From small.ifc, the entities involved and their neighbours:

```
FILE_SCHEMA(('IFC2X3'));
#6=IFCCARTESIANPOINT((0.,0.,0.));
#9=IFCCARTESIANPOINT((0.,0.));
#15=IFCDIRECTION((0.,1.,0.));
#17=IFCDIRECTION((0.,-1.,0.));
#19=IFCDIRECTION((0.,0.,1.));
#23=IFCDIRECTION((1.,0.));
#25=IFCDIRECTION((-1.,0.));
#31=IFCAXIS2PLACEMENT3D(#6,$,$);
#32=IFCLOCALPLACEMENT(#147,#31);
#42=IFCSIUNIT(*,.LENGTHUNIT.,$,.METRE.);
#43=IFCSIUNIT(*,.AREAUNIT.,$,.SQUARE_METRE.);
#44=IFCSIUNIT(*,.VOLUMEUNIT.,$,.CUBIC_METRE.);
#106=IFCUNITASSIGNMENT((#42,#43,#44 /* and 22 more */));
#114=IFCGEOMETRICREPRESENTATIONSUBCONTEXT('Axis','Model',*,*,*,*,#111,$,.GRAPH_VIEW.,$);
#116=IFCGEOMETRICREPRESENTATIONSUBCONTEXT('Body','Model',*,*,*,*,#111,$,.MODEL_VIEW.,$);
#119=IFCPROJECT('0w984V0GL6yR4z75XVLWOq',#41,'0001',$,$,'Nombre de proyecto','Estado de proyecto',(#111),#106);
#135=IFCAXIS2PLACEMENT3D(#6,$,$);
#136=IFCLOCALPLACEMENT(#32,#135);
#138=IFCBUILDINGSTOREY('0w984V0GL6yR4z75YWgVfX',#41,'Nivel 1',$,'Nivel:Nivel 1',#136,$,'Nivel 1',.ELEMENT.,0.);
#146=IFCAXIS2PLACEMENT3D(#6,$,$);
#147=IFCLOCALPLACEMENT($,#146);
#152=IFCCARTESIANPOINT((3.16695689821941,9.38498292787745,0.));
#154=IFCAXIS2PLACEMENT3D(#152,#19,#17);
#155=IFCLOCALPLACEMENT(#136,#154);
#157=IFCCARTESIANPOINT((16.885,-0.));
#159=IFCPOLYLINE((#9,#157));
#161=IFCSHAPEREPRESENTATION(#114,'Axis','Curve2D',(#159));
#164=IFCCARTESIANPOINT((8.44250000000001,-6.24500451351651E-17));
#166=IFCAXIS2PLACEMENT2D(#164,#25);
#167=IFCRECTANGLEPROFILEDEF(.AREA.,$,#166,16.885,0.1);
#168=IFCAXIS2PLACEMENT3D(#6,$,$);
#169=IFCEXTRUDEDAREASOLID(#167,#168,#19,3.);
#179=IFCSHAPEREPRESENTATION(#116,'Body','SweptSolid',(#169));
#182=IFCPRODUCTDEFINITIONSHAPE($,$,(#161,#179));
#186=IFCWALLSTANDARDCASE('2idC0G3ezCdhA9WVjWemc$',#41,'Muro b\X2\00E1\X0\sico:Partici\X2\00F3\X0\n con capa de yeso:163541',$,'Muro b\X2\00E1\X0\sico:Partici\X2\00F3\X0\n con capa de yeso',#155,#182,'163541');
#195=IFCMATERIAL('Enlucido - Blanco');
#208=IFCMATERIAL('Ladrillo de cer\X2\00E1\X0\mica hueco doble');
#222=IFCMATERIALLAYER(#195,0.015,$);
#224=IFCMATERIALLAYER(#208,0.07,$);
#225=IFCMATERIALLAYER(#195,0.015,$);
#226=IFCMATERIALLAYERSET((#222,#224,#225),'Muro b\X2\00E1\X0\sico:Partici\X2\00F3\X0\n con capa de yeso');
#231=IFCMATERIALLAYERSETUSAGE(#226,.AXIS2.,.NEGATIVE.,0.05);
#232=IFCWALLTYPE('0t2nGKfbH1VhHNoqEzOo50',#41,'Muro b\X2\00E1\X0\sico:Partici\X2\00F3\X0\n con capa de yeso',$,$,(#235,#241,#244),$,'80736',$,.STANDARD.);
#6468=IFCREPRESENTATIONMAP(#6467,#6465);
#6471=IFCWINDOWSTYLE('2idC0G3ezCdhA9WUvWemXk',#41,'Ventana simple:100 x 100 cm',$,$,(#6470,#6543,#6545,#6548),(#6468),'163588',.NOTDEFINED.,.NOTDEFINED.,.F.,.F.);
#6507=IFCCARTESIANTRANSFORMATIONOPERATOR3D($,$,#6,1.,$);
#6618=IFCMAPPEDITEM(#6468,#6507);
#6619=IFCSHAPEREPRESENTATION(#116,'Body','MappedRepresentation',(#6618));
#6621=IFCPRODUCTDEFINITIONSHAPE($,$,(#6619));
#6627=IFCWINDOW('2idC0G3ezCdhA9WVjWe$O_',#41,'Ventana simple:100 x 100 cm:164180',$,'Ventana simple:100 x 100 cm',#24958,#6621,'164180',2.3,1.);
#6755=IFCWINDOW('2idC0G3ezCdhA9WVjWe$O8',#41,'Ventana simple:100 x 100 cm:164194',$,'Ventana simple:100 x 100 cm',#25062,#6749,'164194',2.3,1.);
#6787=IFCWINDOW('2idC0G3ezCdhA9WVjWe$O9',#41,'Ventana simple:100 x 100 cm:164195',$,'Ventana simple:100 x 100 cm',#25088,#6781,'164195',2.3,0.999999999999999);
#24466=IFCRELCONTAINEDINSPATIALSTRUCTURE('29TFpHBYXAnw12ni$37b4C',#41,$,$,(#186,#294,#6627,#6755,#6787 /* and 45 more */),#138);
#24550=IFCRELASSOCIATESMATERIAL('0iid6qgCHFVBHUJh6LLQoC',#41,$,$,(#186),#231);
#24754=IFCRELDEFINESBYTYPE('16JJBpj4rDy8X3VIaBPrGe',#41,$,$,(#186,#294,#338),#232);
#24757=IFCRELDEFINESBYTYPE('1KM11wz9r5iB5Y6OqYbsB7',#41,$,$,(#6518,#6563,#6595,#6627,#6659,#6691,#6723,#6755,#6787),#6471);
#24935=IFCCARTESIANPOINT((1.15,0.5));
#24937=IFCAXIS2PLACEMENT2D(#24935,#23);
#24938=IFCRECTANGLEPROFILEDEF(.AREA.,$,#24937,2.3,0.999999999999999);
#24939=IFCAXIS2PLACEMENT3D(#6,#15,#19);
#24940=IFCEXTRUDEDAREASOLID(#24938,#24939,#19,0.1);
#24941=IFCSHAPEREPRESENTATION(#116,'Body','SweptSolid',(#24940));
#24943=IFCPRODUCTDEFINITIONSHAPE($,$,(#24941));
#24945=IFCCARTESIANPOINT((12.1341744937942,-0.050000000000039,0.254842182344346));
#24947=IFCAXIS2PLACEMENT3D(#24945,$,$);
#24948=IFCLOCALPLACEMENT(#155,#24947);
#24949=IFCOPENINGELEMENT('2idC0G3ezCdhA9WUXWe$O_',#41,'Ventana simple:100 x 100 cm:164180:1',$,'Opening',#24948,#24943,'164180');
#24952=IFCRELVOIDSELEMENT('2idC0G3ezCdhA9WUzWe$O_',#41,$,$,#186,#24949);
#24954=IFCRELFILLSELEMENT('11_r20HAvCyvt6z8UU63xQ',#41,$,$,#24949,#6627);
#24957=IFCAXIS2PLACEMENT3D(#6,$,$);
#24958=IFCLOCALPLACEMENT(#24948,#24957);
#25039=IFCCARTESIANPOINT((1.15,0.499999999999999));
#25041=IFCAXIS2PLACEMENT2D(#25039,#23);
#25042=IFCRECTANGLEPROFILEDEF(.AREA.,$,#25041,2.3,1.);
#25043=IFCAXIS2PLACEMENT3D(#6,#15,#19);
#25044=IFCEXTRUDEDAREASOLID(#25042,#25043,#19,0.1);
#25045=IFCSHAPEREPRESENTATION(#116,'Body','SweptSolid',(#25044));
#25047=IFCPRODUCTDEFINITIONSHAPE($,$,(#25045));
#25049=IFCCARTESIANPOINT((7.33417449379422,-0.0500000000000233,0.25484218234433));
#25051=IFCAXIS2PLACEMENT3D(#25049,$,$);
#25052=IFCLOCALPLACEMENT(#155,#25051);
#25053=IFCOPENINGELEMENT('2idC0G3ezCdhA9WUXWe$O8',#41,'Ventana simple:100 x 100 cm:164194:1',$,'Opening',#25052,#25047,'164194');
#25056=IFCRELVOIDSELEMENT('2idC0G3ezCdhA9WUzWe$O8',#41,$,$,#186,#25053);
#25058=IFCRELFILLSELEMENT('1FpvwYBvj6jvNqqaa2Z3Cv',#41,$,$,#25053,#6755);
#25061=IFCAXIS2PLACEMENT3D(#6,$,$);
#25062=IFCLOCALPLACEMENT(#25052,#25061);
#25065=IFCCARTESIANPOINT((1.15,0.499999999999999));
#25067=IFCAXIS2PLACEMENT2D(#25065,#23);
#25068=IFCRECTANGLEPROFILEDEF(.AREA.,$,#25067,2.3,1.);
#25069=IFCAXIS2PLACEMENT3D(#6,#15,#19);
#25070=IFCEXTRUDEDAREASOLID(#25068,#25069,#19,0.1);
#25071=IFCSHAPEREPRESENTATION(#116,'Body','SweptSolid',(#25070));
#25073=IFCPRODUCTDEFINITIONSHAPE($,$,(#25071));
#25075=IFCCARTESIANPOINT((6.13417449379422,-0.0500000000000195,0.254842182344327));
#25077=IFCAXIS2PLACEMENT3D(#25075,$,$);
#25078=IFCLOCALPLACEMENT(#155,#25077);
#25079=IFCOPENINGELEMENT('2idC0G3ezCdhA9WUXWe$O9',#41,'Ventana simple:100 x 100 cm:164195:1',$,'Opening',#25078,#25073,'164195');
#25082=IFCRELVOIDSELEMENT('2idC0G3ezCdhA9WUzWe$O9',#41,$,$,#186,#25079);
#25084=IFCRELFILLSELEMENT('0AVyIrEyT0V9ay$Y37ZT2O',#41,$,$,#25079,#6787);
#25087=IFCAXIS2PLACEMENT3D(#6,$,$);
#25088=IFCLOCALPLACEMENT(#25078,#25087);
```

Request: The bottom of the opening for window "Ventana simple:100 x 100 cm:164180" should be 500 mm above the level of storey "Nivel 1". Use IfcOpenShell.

```python
import numpy as np
import ifcopenshell
import ifcopenshell.api.geometry
import ifcopenshell.geom
import ifcopenshell.util.element
import ifcopenshell.util.placement
import ifcopenshell.util.shape
import ifcopenshell.util.unit

model = ifcopenshell.open("small.ifc")
unit_scale = ifcopenshell.util.unit.calculate_unit_scale(model)

window = model.by_id(6627)
opening = window.FillsVoids[0].RelatingOpeningElement
storey = ifcopenshell.util.element.get_container(window, ifc_class="IfcBuildingStorey")
level = ifcopenshell.util.placement.get_local_placement(storey.ObjectPlacement)[2, 3]

# The opening's origin need not be at the sill, so measure its lowest point.
shape = ifcopenshell.geom.create_shape(ifcopenshell.geom.settings(), opening)
bottom = ifcopenshell.util.shape.get_shape_bottom_elevation(shape, shape.geometry) / unit_scale
dz = level + 0.5 / unit_scale - bottom

shift = np.array([0.0, 0.0, dz])
# The window is placed relative to its opening, so it follows when the opening moves.
matrix = ifcopenshell.util.placement.get_local_placement(opening.ObjectPlacement)
matrix[:3, 3] += shift
ifcopenshell.api.geometry.edit_object_placement(
    model, product=opening, matrix=matrix, is_si=False, should_transform_children=True
)

print(f"moved by {dz * unit_scale:+.3f} m")

model.write("small_edited.ifc")
```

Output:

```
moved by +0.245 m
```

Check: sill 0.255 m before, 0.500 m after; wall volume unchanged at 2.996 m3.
